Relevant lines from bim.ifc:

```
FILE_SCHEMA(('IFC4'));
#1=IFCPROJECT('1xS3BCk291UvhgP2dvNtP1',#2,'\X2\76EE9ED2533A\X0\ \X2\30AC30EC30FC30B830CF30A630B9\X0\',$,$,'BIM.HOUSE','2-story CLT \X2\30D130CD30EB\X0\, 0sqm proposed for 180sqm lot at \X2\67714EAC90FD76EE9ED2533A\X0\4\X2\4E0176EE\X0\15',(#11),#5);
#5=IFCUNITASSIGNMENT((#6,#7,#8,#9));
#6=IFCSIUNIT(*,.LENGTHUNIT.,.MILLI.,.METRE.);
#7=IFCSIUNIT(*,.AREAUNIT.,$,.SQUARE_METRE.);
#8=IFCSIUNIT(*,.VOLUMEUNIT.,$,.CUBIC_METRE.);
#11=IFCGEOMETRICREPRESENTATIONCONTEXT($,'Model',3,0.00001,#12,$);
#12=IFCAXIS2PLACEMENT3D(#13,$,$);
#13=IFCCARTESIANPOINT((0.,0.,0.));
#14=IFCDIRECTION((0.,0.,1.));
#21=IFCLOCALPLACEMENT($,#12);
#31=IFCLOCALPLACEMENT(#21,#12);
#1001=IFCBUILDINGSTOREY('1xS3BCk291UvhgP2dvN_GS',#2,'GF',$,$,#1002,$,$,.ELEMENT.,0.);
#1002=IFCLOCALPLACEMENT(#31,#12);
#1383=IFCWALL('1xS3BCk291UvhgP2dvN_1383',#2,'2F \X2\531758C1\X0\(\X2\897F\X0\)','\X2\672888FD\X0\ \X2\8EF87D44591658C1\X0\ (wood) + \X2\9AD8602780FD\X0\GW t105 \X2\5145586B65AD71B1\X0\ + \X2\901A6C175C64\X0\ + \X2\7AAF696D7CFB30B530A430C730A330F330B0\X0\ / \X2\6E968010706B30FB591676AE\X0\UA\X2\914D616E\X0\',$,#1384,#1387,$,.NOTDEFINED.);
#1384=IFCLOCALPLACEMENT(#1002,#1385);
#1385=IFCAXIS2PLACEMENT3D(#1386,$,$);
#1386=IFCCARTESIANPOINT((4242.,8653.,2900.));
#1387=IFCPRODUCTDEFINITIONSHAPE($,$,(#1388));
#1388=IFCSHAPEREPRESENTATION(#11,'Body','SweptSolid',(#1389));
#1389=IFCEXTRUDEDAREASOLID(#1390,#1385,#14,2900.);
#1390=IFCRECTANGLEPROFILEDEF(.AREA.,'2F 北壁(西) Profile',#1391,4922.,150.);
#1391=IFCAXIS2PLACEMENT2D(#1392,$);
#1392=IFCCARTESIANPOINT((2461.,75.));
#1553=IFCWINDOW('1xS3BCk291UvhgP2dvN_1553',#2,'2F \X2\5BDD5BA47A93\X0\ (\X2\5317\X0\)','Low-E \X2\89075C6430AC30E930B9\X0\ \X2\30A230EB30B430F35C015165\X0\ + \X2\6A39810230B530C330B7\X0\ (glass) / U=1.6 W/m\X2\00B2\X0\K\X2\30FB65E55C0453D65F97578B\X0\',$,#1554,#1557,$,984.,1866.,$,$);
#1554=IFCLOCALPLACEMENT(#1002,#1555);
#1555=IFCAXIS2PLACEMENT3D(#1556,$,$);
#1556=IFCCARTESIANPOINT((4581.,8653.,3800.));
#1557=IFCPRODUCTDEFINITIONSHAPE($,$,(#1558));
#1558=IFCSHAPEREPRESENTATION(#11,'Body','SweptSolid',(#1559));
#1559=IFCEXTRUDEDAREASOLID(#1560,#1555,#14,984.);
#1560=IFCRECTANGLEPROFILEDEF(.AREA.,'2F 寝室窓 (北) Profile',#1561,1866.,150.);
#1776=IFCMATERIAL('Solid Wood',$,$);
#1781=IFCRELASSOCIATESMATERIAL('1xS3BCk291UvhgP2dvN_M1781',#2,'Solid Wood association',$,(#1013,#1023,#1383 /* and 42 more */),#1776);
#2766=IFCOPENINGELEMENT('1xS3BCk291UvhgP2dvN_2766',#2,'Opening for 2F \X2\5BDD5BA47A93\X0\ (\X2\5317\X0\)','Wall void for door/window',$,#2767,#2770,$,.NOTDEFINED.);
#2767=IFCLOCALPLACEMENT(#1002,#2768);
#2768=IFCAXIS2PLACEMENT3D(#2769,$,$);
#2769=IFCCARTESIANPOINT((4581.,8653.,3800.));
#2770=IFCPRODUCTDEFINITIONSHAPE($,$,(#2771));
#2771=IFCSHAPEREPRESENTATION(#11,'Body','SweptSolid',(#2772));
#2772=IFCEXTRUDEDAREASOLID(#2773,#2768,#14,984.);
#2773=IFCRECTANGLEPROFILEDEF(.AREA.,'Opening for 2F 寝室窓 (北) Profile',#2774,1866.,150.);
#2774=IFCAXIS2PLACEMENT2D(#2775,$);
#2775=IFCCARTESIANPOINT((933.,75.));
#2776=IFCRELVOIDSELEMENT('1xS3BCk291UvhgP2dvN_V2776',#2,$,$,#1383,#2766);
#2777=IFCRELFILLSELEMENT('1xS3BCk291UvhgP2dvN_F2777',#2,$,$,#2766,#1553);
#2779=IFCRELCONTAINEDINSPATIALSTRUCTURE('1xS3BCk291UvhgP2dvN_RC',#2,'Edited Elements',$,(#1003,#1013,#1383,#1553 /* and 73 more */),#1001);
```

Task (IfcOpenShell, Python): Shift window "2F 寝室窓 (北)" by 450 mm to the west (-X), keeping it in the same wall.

```python
import ifcopenshell
import ifcopenshell.api.geometry
import ifcopenshell.util.placement
import ifcopenshell.util.unit

model = ifcopenshell.open("bim.ifc")
unit_scale = ifcopenshell.util.unit.calculate_unit_scale(model)

window = model.by_guid("1xS3BCk291UvhgP2dvN_1553")
opening = window.FillsVoids[0].RelatingOpeningElement
wall = opening.VoidsElements[0].RelatingBuildingElement

wall_matrix = ifcopenshell.util.placement.get_local_placement(wall.ObjectPlacement)
shift = wall_matrix[:3, 0] * -0.45 / unit_scale
before = ifcopenshell.util.placement.get_local_placement(window.ObjectPlacement)[:3, 3].copy()

# The window is not placed relative to its opening, so move both.
for product in (opening, window):
    matrix = ifcopenshell.util.placement.get_local_placement(product.ObjectPlacement)
    matrix[:3, 3] += shift
    ifcopenshell.api.geometry.edit_object_placement(model, product=product, matrix=matrix, is_si=False)

after = ifcopenshell.util.placement.get_local_placement(window.ObjectPlacement)[:3, 3]
print("window moved by", (after - before).round(3) + 0.0)

model.write("bim_edited.ifc")
```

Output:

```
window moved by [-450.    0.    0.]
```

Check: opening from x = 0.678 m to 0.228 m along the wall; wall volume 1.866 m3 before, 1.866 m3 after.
